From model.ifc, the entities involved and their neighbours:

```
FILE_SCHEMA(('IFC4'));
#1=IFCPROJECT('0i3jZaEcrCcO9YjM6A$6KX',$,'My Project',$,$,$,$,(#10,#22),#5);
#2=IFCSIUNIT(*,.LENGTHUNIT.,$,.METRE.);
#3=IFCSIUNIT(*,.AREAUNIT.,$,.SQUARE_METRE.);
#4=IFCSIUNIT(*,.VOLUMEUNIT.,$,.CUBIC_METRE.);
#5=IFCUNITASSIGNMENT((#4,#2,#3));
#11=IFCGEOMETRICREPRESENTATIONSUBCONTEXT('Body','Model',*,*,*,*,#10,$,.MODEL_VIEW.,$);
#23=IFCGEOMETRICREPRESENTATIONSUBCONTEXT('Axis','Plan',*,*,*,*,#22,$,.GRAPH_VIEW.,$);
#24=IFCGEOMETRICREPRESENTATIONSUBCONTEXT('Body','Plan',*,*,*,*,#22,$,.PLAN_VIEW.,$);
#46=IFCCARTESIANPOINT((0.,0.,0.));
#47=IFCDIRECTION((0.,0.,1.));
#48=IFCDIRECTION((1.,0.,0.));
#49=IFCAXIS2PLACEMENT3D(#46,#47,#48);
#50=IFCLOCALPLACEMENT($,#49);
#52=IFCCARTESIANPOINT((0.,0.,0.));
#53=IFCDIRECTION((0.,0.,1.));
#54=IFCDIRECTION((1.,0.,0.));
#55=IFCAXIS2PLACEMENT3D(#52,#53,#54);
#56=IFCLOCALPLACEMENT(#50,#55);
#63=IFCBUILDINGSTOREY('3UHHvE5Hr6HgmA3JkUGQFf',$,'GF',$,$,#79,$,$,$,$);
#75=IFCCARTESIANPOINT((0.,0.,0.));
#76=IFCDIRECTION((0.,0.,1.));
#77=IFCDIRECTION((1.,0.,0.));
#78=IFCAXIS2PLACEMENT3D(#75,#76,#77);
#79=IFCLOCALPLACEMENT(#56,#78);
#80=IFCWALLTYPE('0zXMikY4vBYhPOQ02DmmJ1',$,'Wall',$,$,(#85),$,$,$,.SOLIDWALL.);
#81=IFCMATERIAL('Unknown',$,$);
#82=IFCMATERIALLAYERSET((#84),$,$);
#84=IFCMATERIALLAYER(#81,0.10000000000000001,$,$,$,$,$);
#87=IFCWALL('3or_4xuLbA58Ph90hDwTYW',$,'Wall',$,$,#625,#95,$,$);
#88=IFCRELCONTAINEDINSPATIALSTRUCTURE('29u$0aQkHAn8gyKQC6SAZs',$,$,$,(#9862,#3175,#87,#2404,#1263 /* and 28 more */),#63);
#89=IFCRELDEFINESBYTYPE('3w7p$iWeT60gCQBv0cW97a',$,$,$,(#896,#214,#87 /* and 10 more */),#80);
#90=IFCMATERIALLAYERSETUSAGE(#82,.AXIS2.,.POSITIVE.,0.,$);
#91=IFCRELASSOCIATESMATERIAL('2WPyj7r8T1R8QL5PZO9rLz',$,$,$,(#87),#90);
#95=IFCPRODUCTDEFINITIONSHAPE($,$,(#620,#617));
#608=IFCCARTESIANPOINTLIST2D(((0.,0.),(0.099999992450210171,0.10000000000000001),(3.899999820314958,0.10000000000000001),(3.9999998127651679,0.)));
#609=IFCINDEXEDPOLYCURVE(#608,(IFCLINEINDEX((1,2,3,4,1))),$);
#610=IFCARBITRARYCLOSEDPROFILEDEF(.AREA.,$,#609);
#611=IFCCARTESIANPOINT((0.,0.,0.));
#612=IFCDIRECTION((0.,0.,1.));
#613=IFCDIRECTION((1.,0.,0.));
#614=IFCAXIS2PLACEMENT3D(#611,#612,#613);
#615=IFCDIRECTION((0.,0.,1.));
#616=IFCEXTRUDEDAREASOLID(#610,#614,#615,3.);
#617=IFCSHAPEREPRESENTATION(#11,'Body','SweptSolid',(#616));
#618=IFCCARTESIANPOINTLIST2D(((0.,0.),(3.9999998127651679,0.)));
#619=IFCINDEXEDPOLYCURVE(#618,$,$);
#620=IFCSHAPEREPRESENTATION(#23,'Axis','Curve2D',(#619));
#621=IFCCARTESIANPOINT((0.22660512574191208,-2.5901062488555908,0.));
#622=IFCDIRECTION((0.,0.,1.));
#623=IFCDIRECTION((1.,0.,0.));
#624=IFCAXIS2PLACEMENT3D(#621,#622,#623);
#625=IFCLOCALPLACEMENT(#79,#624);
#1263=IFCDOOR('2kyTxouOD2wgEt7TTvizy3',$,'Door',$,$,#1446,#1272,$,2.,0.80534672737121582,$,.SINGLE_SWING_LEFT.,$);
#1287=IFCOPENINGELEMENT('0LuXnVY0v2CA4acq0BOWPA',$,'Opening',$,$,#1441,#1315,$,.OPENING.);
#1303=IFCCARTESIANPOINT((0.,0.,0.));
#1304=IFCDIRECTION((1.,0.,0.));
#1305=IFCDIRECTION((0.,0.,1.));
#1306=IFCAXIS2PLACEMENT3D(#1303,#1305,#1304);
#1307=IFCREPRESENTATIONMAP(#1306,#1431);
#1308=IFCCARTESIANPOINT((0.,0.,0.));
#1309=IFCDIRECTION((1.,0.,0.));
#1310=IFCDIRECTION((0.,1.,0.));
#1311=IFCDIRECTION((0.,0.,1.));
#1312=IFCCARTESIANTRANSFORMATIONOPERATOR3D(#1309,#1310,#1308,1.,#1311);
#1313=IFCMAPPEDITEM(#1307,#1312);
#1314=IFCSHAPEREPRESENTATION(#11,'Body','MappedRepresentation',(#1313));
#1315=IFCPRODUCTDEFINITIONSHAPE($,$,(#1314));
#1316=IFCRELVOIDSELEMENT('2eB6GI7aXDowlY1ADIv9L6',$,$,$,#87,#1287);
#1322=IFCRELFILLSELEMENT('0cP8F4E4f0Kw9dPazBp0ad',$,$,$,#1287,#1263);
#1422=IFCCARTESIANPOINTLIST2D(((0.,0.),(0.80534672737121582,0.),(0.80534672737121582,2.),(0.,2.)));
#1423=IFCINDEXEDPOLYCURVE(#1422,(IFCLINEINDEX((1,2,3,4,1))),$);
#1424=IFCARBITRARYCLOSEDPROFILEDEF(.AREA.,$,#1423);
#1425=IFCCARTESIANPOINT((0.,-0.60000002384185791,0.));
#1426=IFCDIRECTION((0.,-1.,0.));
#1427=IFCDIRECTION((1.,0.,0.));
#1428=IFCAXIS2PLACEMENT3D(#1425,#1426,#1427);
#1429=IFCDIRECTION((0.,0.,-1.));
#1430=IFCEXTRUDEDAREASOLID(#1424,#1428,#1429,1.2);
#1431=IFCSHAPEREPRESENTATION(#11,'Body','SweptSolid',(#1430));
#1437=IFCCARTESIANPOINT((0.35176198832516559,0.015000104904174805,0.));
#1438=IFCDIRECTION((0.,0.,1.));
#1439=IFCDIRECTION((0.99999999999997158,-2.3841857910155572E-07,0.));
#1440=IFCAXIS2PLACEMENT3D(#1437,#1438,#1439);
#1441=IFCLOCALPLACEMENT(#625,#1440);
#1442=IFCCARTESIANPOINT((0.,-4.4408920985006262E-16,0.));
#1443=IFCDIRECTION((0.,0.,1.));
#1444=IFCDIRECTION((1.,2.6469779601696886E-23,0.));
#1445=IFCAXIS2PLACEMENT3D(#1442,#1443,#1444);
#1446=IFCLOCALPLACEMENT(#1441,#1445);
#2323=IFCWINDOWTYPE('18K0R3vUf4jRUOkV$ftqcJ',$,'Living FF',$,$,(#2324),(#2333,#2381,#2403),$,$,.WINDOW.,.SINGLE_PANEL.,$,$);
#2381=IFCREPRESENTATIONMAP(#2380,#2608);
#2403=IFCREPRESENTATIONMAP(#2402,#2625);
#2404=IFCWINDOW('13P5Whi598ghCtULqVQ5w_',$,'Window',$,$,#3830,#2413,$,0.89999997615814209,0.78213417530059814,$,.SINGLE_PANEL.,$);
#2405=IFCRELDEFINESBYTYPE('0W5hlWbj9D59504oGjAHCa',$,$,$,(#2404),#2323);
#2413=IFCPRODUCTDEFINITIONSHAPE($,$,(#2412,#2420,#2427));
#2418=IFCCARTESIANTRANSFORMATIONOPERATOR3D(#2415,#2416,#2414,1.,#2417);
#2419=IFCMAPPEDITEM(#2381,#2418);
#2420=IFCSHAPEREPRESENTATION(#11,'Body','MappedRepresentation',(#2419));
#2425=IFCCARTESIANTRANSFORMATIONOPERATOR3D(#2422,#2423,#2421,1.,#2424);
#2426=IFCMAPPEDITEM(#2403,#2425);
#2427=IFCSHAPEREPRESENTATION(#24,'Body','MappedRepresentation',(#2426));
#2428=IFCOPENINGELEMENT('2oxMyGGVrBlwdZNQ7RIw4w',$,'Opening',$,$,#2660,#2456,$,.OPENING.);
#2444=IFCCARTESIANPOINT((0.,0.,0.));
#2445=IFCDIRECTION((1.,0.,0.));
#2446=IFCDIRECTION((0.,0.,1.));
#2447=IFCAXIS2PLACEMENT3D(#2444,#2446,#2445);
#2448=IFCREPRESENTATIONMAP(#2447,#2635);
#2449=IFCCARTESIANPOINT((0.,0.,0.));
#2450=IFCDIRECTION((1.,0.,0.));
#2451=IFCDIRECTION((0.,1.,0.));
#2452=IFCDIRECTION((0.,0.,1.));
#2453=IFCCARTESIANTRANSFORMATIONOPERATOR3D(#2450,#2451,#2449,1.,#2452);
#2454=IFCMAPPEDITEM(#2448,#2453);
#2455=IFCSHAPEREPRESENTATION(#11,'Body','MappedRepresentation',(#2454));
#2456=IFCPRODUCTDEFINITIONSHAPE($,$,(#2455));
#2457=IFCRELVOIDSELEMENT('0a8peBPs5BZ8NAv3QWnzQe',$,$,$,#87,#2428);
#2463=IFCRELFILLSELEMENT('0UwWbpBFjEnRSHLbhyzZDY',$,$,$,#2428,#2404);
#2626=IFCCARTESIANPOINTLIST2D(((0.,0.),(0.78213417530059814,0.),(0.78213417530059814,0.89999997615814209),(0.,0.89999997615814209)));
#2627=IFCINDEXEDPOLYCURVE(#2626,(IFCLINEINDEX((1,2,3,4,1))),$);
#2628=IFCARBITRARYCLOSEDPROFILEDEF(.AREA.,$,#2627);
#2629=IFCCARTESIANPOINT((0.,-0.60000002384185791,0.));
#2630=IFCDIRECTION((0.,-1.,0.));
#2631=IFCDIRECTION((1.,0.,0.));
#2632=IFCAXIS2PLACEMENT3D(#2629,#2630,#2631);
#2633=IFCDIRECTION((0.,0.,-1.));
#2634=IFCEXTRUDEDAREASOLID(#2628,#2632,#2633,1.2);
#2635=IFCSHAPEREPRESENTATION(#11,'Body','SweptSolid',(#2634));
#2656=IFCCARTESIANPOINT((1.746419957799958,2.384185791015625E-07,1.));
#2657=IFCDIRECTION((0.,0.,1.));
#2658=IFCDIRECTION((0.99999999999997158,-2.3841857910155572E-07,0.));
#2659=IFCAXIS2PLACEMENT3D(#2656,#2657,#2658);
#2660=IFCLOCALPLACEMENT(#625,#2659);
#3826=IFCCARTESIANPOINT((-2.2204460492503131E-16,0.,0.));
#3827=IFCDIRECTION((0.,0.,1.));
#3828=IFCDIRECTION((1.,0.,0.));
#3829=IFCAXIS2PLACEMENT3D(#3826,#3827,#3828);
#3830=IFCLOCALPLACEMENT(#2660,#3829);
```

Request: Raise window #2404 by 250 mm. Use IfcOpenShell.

```python
import numpy as np
import ifcopenshell
import ifcopenshell.api.geometry
import ifcopenshell.util.placement
import ifcopenshell.util.unit

model = ifcopenshell.open("model.ifc")
unit_scale = ifcopenshell.util.unit.calculate_unit_scale(model)

window = model.by_guid("13P5Whi598ghCtULqVQ5w_")
opening = window.FillsVoids[0].RelatingOpeningElement
dz = 0.25

shift = np.array([0.0, 0.0, dz])
# The window is placed relative to its opening, so it follows when the opening moves.
matrix = ifcopenshell.util.placement.get_local_placement(opening.ObjectPlacement)
matrix[:3, 3] += shift
ifcopenshell.api.geometry.edit_object_placement(
    model, product=opening, matrix=matrix, is_si=False, should_transform_children=True
)

print(f"moved by {dz * unit_scale:+.3f} m")

model.write("model_edited.ifc")
```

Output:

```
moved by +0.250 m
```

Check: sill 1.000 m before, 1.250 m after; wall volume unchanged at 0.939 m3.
